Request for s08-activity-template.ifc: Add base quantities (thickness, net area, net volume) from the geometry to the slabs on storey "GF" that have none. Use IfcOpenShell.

First a look at what the model holds.

```python
import ifcopenshell
import ifcopenshell.util.element
import ifcopenshell.util.unit

model = ifcopenshell.open("s08-activity-template.ifc")
print(model.schema)
for unit_type in ("LENGTHUNIT", "AREAUNIT", "VOLUMEUNIT"):
    print(unit_type, ifcopenshell.util.unit.calculate_unit_scale(model, unit_type))
storey = next(s for s in model.by_type("IfcBuildingStorey") if s.Name == "GF")
slabs = [e for e in ifcopenshell.util.element.get_decomposition(storey) if e.is_a("IfcSlab")]
for e in sorted(slabs, key=lambda e: e.id()):
    print(e.id(), e.is_a(), e.Name, list(ifcopenshell.util.element.get_psets(e, qtos_only=True)), sep=" | ")
```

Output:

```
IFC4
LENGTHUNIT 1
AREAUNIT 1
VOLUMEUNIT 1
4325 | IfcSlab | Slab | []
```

```python
import ifcopenshell
import ifcopenshell.api.pset
import ifcopenshell.geom
import ifcopenshell.util.element
import ifcopenshell.util.shape
import ifcopenshell.util.unit

model = ifcopenshell.open("s08-activity-template.ifc")
unit_scale = ifcopenshell.util.unit.calculate_unit_scale(model)
area_scale = ifcopenshell.util.unit.calculate_unit_scale(model, "AREAUNIT")
volume_scale = ifcopenshell.util.unit.calculate_unit_scale(model, "VOLUMEUNIT")
settings = ifcopenshell.geom.settings()

storey = next(s for s in model.by_type("IfcBuildingStorey") if s.Name == "GF")
slabs = [e for e in ifcopenshell.util.element.get_decomposition(storey) if e.is_a("IfcSlab")]

for e in sorted(slabs, key=lambda e: e.id()):
    if ifcopenshell.util.element.get_psets(e, qtos_only=True, should_inherit=False):
        continue
    # Geometry comes back in metres, in the element's own axes.
    shape = ifcopenshell.geom.create_shape(settings, e)
    values = {
        "Width": ifcopenshell.util.shape.get_z(shape.geometry) / unit_scale,
        "NetArea": ifcopenshell.util.shape.get_footprint_area(shape.geometry) / area_scale,
        "NetVolume": ifcopenshell.util.shape.get_volume(shape.geometry) / volume_scale,
    }
    qto = ifcopenshell.api.pset.add_qto(model, product=e, name="Qto_SlabBaseQuantities")
    ifcopenshell.api.pset.edit_qto(model, qto=qto, properties=values)
    print(e.id(), {k: round(v, 3) for k, v in values.items()})

model.write("s08-activity-template_rev.ifc")
```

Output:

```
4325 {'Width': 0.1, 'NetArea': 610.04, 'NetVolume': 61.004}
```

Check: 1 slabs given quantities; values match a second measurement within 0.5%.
